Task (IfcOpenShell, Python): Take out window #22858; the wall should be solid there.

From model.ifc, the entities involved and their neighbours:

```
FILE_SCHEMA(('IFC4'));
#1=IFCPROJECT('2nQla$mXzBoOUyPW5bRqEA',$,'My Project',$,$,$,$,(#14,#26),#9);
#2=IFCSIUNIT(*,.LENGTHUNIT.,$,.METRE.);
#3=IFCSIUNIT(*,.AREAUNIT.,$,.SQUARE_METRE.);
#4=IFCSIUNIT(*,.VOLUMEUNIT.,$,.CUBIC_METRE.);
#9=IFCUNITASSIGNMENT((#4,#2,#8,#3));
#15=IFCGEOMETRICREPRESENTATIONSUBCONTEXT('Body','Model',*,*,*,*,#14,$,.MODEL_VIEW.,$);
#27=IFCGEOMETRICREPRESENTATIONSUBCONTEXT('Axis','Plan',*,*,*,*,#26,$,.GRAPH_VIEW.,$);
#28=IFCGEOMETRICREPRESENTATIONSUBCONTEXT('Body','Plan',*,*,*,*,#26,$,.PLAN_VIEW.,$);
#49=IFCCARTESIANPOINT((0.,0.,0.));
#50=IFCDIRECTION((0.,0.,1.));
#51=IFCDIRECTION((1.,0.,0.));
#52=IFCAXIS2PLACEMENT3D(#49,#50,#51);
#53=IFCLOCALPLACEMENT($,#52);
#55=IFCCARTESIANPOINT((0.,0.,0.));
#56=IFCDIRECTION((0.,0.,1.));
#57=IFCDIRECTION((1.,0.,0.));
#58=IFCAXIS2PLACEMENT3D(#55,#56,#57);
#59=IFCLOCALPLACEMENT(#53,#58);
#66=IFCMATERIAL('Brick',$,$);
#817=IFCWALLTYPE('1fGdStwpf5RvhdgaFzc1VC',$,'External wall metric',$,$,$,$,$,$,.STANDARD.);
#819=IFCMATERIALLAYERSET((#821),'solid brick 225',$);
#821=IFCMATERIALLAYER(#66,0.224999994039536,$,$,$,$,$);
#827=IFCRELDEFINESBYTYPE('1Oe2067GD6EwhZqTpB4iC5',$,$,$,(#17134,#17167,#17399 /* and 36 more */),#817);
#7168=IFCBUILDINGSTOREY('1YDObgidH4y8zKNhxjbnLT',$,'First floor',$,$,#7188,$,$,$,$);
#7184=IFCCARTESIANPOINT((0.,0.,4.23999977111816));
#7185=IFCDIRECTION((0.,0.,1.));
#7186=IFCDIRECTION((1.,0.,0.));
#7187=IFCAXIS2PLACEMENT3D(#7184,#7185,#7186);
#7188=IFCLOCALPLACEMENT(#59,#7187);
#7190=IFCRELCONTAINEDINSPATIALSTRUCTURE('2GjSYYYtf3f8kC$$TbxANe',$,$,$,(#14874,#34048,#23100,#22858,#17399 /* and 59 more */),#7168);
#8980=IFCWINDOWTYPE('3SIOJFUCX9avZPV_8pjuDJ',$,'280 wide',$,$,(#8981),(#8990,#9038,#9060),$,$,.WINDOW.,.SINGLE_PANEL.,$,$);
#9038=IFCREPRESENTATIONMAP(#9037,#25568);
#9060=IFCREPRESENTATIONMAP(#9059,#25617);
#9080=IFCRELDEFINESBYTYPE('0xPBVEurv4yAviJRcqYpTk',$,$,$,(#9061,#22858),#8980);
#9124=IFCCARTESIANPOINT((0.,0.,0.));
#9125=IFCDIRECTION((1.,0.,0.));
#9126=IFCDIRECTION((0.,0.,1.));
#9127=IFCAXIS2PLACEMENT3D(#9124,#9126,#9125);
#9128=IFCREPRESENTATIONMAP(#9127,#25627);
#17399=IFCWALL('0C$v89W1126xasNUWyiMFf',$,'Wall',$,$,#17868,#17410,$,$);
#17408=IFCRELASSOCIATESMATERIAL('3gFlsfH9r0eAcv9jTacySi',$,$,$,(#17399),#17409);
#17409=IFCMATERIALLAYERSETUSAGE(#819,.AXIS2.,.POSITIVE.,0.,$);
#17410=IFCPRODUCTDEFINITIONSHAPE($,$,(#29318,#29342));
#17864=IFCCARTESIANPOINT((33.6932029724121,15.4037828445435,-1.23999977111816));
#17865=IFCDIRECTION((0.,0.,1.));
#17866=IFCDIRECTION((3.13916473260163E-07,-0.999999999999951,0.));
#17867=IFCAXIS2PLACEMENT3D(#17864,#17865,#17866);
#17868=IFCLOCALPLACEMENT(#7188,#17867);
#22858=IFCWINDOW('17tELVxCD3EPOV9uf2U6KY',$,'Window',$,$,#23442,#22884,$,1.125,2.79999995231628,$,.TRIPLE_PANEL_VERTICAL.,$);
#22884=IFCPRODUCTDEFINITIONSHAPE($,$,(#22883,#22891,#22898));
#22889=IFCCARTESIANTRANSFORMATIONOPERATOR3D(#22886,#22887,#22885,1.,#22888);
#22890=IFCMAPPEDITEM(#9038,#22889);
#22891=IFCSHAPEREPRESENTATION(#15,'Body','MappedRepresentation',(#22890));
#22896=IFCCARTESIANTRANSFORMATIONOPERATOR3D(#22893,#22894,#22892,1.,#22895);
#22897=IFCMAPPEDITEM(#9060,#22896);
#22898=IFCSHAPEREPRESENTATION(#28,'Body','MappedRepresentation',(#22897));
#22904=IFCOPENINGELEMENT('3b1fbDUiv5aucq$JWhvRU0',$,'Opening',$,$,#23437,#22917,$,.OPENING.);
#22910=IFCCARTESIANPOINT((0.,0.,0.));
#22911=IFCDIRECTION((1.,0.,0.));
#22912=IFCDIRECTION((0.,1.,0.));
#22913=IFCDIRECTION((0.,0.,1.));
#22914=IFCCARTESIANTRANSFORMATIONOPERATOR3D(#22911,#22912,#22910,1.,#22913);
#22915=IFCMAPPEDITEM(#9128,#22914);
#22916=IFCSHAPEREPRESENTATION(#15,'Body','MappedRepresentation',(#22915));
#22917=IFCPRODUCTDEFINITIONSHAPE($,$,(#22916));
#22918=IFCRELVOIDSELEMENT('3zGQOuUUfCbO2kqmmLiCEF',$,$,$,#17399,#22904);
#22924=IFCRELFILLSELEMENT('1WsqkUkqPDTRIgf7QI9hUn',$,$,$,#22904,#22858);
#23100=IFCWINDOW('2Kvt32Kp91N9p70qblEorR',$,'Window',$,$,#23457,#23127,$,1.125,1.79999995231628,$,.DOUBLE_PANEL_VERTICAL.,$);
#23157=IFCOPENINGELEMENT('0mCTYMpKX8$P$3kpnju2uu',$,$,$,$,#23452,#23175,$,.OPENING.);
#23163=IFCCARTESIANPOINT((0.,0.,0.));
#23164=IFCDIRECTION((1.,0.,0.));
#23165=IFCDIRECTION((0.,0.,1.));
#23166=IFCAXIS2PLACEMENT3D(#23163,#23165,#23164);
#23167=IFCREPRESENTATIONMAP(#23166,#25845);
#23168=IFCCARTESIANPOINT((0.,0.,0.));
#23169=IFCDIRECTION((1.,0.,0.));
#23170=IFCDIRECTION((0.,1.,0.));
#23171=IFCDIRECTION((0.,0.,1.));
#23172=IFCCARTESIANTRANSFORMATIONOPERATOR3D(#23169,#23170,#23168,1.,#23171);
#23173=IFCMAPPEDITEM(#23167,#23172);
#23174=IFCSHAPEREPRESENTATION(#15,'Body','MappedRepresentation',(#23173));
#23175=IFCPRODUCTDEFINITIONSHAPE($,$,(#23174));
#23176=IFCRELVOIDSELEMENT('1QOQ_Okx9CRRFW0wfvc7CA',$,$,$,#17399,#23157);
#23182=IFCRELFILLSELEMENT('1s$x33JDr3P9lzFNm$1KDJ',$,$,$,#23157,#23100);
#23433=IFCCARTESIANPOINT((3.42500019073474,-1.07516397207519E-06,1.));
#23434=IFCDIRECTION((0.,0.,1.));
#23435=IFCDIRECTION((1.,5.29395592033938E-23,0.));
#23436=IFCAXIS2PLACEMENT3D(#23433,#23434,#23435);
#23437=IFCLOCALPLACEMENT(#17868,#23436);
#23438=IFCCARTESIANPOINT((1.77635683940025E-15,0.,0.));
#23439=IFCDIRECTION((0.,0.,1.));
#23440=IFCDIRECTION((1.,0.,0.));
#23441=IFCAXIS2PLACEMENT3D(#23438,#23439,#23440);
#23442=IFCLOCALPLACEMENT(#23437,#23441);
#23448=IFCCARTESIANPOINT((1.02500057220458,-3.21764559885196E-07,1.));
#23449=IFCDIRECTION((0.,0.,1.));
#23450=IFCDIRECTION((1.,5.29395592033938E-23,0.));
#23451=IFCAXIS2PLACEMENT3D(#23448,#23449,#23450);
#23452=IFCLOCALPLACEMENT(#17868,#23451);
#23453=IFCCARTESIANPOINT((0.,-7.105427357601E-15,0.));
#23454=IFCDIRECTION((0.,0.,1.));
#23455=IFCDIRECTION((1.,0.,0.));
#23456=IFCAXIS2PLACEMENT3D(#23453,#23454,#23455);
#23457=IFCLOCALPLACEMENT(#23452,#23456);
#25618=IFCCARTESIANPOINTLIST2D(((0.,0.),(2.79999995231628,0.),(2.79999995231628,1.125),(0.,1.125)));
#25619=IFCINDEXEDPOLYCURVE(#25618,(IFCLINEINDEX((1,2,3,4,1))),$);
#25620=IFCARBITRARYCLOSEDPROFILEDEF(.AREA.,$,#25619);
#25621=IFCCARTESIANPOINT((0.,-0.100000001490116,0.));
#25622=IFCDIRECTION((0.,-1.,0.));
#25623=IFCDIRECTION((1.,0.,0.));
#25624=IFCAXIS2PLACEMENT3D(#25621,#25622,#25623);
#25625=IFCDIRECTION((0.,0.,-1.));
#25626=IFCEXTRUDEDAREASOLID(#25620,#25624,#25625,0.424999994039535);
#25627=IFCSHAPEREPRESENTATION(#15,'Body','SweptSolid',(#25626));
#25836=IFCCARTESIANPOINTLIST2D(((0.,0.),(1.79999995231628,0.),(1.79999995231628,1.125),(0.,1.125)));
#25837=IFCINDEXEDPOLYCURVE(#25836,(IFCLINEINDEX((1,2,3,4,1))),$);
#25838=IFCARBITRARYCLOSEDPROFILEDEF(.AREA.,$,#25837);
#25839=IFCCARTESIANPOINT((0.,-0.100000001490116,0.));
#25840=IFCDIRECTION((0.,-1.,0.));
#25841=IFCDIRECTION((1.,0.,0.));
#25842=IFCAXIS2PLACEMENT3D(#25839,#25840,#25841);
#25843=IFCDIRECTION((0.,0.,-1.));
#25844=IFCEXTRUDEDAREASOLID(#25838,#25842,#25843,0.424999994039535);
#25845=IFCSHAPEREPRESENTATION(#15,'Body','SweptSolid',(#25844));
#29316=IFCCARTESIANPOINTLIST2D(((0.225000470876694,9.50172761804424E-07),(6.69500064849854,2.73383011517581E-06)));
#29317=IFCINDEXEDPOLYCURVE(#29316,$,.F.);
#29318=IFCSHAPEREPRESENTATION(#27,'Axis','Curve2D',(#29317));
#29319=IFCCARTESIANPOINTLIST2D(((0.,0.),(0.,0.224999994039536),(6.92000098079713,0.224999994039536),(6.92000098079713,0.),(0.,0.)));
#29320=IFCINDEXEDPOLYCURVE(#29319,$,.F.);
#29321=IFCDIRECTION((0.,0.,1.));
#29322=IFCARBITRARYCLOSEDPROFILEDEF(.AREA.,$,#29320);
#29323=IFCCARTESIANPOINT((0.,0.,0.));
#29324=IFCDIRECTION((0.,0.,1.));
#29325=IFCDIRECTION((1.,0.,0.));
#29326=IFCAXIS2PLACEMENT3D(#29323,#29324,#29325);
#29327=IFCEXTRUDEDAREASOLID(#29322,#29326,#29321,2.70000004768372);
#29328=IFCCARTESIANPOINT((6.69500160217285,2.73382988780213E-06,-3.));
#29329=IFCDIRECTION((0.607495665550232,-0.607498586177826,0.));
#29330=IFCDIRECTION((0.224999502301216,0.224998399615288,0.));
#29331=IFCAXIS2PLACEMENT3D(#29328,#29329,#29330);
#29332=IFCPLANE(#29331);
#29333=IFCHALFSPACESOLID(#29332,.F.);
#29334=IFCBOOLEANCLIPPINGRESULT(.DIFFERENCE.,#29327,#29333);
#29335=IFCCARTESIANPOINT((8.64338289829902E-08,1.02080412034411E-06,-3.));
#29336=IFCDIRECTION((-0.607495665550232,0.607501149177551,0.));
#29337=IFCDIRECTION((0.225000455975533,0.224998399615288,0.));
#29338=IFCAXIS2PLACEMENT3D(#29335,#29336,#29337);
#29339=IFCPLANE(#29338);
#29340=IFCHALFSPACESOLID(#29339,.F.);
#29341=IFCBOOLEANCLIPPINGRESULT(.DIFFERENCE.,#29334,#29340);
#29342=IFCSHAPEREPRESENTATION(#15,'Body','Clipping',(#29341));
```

```python
import ifcopenshell
import ifcopenshell.api.feature
import ifcopenshell.api.root
import ifcopenshell.geom
import ifcopenshell.util.shape

model = ifcopenshell.open("model.ifc")
settings = ifcopenshell.geom.settings()


def volume(element):
    """Net volume in cubic metres, openings subtracted."""
    shape = ifcopenshell.geom.create_shape(settings, element)
    return ifcopenshell.util.shape.get_volume(shape.geometry)


window = model.by_id(22858)
opening = window.FillsVoids[0].RelatingOpeningElement
wall = opening.VoidsElements[0].RelatingBuildingElement
before = volume(wall)

ifcopenshell.api.root.remove_product(model, product=window)
ifcopenshell.api.feature.remove_feature(model, feature=opening)

after = volume(wall)

print(f"wall volume {before:.3f} -> {after:.3f} m3")

model.write("model_updated.ifc")
```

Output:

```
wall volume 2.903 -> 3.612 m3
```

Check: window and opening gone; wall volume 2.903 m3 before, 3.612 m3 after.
